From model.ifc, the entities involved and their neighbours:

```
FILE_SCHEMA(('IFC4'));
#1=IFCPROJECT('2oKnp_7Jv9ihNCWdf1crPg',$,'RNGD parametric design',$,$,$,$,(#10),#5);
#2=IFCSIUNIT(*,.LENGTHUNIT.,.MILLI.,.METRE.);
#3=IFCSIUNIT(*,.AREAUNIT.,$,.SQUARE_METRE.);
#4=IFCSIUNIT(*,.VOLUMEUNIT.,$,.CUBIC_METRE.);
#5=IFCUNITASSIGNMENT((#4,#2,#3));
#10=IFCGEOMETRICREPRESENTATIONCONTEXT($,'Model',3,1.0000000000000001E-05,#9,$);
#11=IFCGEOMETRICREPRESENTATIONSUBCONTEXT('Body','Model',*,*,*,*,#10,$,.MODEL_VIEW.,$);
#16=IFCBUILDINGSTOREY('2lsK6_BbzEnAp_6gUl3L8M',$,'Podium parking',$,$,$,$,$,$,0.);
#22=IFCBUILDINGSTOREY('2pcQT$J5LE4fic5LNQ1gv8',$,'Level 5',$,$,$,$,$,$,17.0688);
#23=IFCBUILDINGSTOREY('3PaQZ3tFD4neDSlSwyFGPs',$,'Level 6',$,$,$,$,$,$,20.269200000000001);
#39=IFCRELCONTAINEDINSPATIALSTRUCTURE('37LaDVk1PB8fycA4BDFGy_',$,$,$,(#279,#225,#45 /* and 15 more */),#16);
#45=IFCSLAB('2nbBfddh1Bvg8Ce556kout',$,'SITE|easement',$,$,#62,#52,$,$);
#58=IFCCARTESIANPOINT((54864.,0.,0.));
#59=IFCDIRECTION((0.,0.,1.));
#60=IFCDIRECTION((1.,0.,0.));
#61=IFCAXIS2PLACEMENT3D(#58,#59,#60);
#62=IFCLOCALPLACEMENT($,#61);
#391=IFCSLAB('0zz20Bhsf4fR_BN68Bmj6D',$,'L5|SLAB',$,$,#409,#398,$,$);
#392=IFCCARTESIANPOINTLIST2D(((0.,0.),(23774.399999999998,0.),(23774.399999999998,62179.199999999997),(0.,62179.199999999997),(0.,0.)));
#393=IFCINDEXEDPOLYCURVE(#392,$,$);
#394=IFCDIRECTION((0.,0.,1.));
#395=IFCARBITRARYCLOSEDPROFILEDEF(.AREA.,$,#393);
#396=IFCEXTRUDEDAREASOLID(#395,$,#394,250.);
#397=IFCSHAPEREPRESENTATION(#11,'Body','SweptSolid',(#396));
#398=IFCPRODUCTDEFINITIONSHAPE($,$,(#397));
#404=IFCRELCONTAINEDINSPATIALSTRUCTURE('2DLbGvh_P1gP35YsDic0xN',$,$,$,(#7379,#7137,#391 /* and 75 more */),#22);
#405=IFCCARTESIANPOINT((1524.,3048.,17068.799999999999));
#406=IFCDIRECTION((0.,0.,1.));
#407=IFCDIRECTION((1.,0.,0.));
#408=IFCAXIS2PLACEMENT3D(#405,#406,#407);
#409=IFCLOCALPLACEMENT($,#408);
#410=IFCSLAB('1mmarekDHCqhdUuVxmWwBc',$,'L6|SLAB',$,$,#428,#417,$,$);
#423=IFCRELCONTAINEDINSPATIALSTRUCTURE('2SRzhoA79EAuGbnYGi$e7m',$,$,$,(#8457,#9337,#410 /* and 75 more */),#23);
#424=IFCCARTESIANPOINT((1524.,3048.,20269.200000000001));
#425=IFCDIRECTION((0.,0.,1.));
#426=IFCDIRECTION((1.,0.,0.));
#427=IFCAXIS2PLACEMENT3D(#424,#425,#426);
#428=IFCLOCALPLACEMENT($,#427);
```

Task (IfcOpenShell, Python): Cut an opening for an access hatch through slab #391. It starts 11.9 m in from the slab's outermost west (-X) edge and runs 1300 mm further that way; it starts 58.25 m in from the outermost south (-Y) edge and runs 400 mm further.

```python
import numpy as np
import ifcopenshell
import ifcopenshell.api.feature
import ifcopenshell.api.geometry
import ifcopenshell.api.root
import ifcopenshell.geom
import ifcopenshell.util.placement
import ifcopenshell.util.representation
import ifcopenshell.util.shape
import ifcopenshell.util.unit

model = ifcopenshell.open("model.ifc")
unit_scale = ifcopenshell.util.unit.calculate_unit_scale(model)
settings = ifcopenshell.geom.settings()


def volume(element):
    """Net volume in cubic metres, openings subtracted."""
    shape = ifcopenshell.geom.create_shape(settings, element)
    return ifcopenshell.util.shape.get_volume(shape.geometry)


slab = model.by_guid("0zz20Bhsf4fR_BN68Bmj6D")
before = volume(slab)

# Extent in the slab's own axes, in metres. The edges named are its -X and -Y sides.
slab_shape = ifcopenshell.geom.create_shape(settings, slab)
vertices = ifcopenshell.util.shape.get_vertices(slab_shape.geometry)
x_min, y_min, bottom = vertices.min(axis=0)
top = vertices[:, 2].max()

opening = ifcopenshell.api.root.create_entity(model, ifc_class="IfcOpeningElement", name="Access hatch opening", predefined_type="OPENING")
context = ifcopenshell.util.representation.get_context(model, "Model", "Body", "MODEL_VIEW")
width, depth = 1.3, 0.4
outline = [(0.0, 0.0), (width, 0.0), (width, depth), (0.0, depth), (0.0, 0.0)]
# Overshoot both faces by 50 mm so the cut is clean.
shape = ifcopenshell.api.geometry.add_slab_representation(
    model, context=context, depth=top - bottom + 0.1, polyline=outline
)
ifcopenshell.api.geometry.assign_representation(model, product=opening, representation=shape)

matrix = ifcopenshell.util.placement.get_local_placement(slab.ObjectPlacement)
matrix[:, 3] = matrix @ np.append(np.array([x_min + 11.9, y_min + 58.25, bottom - 0.05]) / unit_scale, 1.0)
ifcopenshell.api.geometry.edit_object_placement(model, product=opening, matrix=matrix, is_si=False)
ifcopenshell.api.feature.add_feature(model, feature=opening, element=slab)

after = volume(slab)

print(f"slab volume {before:.3f} -> {after:.3f} m3")

model.write("model-out.ifc")
```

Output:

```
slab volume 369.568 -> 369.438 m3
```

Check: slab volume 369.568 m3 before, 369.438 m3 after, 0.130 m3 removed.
